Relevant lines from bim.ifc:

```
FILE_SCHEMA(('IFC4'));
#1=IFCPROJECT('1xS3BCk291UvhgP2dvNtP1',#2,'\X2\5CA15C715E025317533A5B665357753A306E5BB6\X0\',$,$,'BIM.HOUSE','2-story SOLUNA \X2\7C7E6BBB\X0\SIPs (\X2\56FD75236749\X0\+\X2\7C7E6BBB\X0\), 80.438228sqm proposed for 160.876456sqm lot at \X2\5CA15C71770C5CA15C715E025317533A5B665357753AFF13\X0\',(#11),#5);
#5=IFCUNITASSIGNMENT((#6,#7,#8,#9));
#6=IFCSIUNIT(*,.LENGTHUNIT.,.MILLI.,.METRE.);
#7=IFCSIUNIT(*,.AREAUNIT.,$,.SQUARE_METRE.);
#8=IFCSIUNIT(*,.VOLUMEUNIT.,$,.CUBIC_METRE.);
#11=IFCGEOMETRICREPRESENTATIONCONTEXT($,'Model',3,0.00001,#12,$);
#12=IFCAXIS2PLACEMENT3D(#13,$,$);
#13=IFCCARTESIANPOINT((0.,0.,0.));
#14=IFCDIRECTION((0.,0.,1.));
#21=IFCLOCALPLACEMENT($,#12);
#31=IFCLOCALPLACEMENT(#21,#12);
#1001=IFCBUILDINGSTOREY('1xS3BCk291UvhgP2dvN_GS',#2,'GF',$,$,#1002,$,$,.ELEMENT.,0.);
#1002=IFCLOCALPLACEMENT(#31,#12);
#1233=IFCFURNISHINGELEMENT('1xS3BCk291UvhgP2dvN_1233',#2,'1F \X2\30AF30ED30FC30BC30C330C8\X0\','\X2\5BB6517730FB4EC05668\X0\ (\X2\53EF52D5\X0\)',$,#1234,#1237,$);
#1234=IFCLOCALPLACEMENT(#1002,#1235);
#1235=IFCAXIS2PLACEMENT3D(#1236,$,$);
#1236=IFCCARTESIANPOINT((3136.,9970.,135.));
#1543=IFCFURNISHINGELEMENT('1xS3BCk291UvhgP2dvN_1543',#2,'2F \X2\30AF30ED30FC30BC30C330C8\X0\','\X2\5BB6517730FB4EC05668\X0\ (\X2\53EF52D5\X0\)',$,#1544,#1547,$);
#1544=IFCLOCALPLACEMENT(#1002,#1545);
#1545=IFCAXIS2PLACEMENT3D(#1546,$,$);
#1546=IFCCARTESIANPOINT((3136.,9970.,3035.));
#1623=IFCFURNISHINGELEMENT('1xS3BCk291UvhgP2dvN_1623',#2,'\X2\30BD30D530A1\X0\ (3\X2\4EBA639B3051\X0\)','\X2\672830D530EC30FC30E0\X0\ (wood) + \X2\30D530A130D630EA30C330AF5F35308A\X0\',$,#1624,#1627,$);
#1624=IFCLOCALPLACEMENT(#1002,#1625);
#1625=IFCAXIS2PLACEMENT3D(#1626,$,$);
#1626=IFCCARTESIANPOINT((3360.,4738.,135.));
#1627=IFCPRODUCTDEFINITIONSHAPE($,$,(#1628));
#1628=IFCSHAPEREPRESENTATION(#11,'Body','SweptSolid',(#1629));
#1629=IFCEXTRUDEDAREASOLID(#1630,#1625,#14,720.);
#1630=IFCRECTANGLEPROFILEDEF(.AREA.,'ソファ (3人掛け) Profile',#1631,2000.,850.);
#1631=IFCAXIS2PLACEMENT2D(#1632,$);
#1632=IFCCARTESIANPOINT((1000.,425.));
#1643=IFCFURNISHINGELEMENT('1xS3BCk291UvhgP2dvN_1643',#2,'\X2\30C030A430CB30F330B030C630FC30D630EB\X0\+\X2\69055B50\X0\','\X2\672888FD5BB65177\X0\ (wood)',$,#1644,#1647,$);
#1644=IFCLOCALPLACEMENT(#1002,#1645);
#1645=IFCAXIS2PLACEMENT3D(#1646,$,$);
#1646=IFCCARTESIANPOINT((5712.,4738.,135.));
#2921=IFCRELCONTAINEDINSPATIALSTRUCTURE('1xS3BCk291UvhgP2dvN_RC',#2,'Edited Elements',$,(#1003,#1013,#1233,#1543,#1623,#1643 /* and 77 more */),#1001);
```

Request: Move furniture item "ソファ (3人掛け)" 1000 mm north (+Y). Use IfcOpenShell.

```python
import ifcopenshell
import ifcopenshell.api.geometry
import ifcopenshell.util.placement
import ifcopenshell.util.unit

model = ifcopenshell.open("bim.ifc")
unit_scale = ifcopenshell.util.unit.calculate_unit_scale(model)

item = model.by_guid("1xS3BCk291UvhgP2dvN_1623")
matrix = ifcopenshell.util.placement.get_local_placement(item.ObjectPlacement)
matrix[1, 3] += 1 / unit_scale
ifcopenshell.api.geometry.edit_object_placement(model, product=item, matrix=matrix, is_si=False)

print(ifcopenshell.util.placement.get_local_placement(item.ObjectPlacement).round(3) + 0.0)

model.write("bim_rev.ifc")
```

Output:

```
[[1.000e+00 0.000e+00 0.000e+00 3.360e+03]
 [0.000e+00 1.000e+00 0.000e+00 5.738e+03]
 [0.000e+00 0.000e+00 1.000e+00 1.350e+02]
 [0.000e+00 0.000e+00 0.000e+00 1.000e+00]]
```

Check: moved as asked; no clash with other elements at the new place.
